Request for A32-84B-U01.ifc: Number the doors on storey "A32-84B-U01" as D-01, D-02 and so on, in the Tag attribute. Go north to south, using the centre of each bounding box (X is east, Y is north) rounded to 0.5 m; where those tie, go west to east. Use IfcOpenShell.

First a look at what the model holds.

```python
import ifcopenshell
import ifcopenshell.util.element
import ifcopenshell.util.placement

model = ifcopenshell.open("A32-84B-U01.ifc")
print(model.schema)
storey = next(s for s in model.by_type("IfcBuildingStorey") if s.Name == "A32-84B-U01")
doors = [e for e in ifcopenshell.util.element.get_decomposition(storey) if e.is_a("IfcDoor")]
for e in sorted(doors, key=lambda e: e.id()):
    origin = ifcopenshell.util.placement.get_local_placement(e.ObjectPlacement)[:3, 3]
    print(e.id(), e.Tag, e.Name, origin.round(2) + 0.0, sep=" | ")
```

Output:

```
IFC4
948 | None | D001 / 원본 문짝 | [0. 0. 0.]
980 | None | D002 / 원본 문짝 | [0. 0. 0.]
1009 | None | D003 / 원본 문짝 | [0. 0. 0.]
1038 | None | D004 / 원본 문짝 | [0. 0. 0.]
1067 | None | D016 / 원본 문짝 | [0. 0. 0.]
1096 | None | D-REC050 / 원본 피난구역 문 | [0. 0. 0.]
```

```python
import ifcopenshell
import ifcopenshell.geom
import ifcopenshell.util.element
import ifcopenshell.util.shape

model = ifcopenshell.open("A32-84B-U01.ifc")
settings = ifcopenshell.geom.settings()
settings.set("use-world-coords", True)


def centre(element):
    shape = ifcopenshell.geom.create_shape(settings, element)
    return ifcopenshell.util.shape.get_bbox_centroid(shape.geometry)


storey = next(s for s in model.by_type("IfcBuildingStorey") if s.Name == "A32-84B-U01")
doors = [e for e in ifcopenshell.util.element.get_decomposition(storey) if e.is_a("IfcDoor")]

# Insertion points can sit at a corner or the storey origin, so sort by the geometry (in metres).
centres = {e: centre(e) for e in doors}
doors.sort(key=lambda e: (-round(centres[e][1] / 0.5), centres[e][0]))

for i, e in enumerate(doors, start=1):
    number = f"D-{i:02d}"
    e.Tag = number
    print(e.id(), number)

model.write("A32-84B-U01_rev.ifc")
```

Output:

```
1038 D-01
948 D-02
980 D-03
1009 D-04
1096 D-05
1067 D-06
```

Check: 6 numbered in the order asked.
